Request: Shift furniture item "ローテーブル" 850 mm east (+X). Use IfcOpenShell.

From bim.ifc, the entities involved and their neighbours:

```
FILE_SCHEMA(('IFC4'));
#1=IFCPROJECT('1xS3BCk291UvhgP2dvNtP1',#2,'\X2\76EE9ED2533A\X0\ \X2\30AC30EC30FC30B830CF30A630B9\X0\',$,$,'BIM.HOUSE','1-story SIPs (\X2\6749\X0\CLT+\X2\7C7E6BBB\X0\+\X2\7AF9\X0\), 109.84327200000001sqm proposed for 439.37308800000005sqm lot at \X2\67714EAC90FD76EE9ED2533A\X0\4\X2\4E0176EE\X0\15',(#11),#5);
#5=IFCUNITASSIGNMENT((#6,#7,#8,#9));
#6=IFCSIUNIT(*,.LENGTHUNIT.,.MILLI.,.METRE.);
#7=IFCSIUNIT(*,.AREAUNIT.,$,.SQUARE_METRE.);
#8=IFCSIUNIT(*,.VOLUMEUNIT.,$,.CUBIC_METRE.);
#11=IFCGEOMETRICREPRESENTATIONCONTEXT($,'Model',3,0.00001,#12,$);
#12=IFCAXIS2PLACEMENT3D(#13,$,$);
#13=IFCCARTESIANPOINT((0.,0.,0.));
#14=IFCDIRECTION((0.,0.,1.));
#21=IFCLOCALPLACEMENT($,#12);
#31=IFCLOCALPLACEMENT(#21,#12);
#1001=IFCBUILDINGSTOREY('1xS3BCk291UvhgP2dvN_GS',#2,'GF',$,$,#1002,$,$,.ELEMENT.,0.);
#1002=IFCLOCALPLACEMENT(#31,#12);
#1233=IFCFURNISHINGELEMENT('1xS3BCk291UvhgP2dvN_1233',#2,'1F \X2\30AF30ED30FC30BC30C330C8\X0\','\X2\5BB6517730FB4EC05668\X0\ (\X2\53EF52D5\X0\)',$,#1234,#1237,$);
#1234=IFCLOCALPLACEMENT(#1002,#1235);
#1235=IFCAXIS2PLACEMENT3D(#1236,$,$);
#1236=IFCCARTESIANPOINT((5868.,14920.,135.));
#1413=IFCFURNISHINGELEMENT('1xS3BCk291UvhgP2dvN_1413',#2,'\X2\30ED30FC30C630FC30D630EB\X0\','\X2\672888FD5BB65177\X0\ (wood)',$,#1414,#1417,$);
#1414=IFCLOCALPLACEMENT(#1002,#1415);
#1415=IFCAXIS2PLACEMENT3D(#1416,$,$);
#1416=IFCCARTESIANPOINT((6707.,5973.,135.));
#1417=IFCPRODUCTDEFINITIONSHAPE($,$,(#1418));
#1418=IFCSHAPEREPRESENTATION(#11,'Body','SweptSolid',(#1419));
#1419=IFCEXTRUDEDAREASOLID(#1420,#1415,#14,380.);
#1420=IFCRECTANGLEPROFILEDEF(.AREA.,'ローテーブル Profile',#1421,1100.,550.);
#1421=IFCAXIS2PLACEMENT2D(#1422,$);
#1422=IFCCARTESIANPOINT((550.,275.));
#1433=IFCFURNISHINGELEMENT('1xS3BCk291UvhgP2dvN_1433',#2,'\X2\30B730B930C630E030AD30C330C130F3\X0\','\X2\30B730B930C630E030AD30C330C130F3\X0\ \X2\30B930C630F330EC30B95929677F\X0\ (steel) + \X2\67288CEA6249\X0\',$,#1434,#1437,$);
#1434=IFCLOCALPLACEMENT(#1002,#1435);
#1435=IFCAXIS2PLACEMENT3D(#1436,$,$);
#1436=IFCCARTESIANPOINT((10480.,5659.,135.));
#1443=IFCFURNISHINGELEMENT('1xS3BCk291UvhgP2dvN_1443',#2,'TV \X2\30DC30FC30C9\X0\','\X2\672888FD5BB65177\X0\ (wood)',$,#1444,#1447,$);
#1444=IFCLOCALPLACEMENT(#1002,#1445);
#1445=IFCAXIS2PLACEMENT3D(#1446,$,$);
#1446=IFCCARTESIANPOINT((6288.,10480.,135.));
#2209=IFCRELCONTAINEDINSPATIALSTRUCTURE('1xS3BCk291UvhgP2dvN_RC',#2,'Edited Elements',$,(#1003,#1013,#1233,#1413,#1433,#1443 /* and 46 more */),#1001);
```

```python
import ifcopenshell
import ifcopenshell.api.geometry
import ifcopenshell.util.placement
import ifcopenshell.util.unit

model = ifcopenshell.open("bim.ifc")
unit_scale = ifcopenshell.util.unit.calculate_unit_scale(model)

item = model.by_guid("1xS3BCk291UvhgP2dvN_1413")
matrix = ifcopenshell.util.placement.get_local_placement(item.ObjectPlacement)
matrix[0, 3] += 0.85 / unit_scale
ifcopenshell.api.geometry.edit_object_placement(model, product=item, matrix=matrix, is_si=False)

print(ifcopenshell.util.placement.get_local_placement(item.ObjectPlacement).round(3) + 0.0)

model.write("bim_edited.ifc")
```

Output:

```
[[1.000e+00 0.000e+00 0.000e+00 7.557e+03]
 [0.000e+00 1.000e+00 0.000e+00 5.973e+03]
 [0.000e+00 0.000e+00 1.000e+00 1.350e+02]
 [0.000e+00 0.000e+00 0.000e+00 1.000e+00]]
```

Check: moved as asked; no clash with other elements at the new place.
